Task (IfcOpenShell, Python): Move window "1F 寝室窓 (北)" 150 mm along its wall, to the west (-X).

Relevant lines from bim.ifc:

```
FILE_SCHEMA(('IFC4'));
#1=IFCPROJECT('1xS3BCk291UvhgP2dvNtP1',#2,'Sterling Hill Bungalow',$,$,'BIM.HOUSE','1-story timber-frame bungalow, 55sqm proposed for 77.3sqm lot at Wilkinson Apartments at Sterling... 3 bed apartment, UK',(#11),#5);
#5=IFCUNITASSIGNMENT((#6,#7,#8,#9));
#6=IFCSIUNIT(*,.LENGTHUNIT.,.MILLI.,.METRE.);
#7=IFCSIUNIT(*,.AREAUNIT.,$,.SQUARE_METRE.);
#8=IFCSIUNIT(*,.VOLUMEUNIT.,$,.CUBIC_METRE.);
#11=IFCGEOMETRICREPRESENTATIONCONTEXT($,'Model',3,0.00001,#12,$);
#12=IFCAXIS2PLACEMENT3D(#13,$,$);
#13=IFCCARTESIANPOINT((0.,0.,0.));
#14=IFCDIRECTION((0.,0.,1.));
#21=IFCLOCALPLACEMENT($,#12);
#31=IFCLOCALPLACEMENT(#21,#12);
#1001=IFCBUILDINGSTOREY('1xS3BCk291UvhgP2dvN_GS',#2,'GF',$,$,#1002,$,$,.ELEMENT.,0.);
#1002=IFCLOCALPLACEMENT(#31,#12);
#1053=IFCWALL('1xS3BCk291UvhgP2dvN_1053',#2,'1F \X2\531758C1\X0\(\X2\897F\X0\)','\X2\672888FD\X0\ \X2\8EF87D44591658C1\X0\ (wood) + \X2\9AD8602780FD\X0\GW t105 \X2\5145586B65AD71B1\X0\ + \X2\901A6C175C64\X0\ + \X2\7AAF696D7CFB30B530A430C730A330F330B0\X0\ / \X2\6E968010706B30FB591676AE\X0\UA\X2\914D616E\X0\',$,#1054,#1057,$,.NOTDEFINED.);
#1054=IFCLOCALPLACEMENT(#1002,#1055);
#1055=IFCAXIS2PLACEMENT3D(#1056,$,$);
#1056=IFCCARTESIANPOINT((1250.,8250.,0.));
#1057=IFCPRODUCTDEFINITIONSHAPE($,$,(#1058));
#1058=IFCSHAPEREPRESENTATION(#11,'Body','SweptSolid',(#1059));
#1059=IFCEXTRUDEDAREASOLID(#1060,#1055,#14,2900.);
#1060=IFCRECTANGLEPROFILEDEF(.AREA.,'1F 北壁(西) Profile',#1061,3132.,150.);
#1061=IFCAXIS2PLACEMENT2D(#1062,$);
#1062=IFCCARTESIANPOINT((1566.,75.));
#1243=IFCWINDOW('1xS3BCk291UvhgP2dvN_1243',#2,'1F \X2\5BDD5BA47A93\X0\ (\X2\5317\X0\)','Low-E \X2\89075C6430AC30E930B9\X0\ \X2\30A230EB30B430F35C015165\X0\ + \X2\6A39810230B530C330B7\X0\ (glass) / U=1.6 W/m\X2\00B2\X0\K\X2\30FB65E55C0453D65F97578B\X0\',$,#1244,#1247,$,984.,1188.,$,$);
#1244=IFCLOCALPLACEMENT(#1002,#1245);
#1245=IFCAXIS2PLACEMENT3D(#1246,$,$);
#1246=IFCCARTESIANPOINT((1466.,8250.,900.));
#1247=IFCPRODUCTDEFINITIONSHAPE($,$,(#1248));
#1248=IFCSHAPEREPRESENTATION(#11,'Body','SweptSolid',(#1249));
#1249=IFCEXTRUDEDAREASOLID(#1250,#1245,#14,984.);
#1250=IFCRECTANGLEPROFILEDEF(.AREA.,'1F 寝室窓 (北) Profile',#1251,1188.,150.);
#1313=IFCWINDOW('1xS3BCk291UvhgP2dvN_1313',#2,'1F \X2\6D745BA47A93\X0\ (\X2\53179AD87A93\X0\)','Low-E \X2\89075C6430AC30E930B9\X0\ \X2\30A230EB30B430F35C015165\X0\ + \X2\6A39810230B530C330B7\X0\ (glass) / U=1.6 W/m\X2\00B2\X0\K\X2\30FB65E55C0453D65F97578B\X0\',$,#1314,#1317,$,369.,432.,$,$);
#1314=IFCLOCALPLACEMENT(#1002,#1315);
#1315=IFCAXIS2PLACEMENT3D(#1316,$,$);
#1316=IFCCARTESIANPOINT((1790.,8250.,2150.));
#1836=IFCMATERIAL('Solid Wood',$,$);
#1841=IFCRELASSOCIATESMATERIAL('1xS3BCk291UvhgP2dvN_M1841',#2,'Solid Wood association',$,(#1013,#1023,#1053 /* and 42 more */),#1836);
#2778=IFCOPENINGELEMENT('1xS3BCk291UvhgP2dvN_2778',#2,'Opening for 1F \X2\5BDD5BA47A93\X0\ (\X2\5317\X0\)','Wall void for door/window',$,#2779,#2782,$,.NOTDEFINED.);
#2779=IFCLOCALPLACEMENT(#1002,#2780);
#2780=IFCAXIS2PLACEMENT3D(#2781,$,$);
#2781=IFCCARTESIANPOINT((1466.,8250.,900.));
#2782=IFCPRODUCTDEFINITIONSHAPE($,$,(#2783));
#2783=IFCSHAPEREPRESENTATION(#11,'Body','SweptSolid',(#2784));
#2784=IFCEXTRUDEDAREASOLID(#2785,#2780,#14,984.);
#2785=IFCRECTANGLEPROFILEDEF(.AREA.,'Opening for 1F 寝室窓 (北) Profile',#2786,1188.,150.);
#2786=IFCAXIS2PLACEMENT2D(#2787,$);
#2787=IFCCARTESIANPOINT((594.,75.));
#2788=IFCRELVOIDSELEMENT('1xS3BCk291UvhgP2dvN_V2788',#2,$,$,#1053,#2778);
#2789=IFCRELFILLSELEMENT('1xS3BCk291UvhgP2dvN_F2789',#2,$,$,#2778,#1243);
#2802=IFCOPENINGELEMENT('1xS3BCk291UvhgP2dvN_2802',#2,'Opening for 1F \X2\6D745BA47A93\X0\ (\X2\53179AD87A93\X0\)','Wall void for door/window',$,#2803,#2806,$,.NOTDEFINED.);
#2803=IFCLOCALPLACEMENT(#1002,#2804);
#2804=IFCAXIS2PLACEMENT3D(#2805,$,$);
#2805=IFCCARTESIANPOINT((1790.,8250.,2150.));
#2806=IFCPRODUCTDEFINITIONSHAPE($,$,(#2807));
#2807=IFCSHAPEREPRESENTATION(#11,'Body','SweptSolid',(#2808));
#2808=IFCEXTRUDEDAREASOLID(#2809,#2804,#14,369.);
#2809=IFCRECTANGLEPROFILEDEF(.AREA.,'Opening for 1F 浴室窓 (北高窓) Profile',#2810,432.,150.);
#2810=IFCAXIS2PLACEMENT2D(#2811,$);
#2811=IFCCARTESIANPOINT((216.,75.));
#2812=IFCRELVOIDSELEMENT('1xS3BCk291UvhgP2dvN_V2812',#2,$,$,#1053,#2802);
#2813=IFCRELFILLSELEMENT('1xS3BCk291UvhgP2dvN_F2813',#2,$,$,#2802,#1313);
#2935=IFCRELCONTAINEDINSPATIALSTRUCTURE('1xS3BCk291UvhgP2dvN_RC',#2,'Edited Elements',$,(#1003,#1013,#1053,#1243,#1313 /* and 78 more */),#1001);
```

```python
import ifcopenshell
import ifcopenshell.api.geometry
import ifcopenshell.util.placement
import ifcopenshell.util.unit

model = ifcopenshell.open("bim.ifc")
unit_scale = ifcopenshell.util.unit.calculate_unit_scale(model)

window = model.by_guid("1xS3BCk291UvhgP2dvN_1243")
opening = window.FillsVoids[0].RelatingOpeningElement
wall = opening.VoidsElements[0].RelatingBuildingElement

wall_matrix = ifcopenshell.util.placement.get_local_placement(wall.ObjectPlacement)
shift = wall_matrix[:3, 0] * -0.15 / unit_scale
before = ifcopenshell.util.placement.get_local_placement(window.ObjectPlacement)[:3, 3].copy()

# The window is not placed relative to its opening, so move both.
for product in (opening, window):
    matrix = ifcopenshell.util.placement.get_local_placement(product.ObjectPlacement)
    matrix[:3, 3] += shift
    ifcopenshell.api.geometry.edit_object_placement(model, product=product, matrix=matrix, is_si=False)

after = ifcopenshell.util.placement.get_local_placement(window.ObjectPlacement)[:3, 3]
print("window moved by", (after - before).round(3) + 0.0)

model.write("bim_v2.ifc")
```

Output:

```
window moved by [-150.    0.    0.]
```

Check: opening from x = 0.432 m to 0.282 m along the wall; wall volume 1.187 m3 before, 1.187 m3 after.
